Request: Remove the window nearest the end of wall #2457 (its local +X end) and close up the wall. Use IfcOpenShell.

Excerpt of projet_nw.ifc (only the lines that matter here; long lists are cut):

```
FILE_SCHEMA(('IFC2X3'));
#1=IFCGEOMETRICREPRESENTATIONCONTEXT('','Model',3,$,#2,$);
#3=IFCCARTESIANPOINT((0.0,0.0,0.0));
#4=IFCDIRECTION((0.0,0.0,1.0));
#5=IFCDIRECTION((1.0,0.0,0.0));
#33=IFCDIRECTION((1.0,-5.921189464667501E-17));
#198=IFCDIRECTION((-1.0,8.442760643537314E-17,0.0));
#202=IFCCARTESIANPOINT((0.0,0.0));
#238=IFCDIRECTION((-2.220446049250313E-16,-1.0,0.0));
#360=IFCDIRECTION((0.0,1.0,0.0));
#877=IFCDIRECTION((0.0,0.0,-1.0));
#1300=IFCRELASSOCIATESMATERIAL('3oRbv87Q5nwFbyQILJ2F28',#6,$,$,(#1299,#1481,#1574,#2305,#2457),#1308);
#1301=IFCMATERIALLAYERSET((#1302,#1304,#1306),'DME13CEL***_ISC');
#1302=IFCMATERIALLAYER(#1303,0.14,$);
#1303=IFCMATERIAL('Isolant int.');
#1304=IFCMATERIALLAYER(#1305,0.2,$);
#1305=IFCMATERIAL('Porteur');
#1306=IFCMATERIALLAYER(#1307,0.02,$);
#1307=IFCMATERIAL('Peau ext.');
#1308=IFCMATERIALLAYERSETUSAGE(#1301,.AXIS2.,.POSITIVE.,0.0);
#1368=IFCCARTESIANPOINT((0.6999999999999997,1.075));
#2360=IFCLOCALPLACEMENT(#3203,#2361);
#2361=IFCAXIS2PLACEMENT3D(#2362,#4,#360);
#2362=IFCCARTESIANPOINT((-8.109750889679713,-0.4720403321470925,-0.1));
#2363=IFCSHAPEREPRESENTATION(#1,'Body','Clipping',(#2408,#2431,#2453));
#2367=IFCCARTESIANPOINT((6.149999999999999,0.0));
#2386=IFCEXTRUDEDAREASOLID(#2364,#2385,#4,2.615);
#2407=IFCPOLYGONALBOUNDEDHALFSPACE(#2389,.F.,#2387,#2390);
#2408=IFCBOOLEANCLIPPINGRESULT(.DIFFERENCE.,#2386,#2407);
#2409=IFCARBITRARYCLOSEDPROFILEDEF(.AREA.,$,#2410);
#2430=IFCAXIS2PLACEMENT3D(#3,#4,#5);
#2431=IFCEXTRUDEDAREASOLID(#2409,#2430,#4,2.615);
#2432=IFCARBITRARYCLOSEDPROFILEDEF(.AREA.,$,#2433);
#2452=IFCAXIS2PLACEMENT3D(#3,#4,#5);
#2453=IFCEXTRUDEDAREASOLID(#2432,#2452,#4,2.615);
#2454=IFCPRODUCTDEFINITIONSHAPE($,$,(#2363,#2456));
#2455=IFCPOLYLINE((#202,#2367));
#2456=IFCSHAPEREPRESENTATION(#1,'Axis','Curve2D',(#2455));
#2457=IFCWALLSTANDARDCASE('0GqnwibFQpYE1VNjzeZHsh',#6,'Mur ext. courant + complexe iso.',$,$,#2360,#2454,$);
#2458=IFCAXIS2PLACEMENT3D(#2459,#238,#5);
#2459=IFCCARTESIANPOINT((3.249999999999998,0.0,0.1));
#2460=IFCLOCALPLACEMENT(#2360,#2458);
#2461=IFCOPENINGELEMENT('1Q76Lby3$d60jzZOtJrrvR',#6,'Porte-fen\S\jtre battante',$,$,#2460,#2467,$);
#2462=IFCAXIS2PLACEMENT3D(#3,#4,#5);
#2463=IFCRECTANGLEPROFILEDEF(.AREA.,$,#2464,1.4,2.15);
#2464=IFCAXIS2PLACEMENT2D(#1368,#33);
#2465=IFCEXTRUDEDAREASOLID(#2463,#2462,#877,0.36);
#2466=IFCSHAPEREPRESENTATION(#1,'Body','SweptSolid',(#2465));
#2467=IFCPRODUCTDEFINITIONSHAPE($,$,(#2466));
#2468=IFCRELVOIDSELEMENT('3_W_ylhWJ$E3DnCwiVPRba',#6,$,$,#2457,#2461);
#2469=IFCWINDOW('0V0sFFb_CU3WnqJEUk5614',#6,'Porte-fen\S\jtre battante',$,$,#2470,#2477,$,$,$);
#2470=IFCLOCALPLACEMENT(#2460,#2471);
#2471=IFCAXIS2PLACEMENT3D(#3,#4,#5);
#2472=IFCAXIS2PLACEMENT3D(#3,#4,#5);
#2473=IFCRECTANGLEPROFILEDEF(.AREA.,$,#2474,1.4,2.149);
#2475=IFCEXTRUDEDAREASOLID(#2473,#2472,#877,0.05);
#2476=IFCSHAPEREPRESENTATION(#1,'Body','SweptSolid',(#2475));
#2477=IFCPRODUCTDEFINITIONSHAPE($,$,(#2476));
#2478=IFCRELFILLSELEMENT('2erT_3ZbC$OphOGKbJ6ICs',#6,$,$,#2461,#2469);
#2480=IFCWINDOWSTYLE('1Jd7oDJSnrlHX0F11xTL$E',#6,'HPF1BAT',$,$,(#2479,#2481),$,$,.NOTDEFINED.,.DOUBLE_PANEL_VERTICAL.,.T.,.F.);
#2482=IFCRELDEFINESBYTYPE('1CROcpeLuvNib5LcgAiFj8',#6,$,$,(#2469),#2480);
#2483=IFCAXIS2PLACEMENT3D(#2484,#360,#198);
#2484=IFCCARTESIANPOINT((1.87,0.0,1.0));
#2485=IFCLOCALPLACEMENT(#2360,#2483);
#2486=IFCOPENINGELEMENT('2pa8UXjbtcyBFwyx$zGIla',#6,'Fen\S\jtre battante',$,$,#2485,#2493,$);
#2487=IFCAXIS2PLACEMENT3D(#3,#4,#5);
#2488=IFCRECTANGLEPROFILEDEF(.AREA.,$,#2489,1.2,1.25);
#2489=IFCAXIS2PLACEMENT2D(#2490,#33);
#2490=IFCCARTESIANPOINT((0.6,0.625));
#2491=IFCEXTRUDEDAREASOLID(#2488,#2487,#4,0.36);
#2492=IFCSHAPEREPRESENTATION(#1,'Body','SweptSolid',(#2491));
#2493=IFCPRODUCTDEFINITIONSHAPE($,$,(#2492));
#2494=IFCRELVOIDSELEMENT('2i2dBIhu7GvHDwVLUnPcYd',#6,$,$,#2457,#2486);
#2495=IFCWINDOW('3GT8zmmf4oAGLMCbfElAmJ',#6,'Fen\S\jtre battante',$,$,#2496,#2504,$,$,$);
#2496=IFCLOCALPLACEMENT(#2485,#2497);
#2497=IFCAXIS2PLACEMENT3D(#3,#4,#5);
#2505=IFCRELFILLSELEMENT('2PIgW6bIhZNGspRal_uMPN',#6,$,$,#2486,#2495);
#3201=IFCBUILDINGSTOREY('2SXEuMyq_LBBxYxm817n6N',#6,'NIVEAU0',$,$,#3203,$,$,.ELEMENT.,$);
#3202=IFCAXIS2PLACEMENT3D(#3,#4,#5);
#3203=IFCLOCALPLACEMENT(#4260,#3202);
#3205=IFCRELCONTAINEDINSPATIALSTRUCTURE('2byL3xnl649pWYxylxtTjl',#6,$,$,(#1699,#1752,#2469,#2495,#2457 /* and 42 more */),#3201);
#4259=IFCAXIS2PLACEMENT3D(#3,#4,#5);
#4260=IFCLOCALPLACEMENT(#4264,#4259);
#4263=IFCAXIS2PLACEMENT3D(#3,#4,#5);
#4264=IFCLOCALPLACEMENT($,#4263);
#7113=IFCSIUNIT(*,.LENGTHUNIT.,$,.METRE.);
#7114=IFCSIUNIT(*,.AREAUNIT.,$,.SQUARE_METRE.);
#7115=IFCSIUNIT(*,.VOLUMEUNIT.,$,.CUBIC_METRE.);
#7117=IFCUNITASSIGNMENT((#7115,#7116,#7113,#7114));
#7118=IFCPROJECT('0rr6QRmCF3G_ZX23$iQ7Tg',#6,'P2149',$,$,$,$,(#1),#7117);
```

```python
import ifcopenshell
import ifcopenshell.api.feature
import ifcopenshell.api.root
import ifcopenshell.geom
import ifcopenshell.util.shape

model = ifcopenshell.open("projet_nw.ifc")
settings = ifcopenshell.geom.settings()


def volume(element):
    """Net volume in cubic metres, openings subtracted."""
    shape = ifcopenshell.geom.create_shape(settings, element)
    return ifcopenshell.util.shape.get_volume(shape.geometry)


window = model.by_guid("0V0sFFb_CU3WnqJEUk5614")
opening = window.FillsVoids[0].RelatingOpeningElement
wall = opening.VoidsElements[0].RelatingBuildingElement
before = volume(wall)

ifcopenshell.api.root.remove_product(model, product=window)
ifcopenshell.api.feature.remove_feature(model, feature=opening)

after = volume(wall)

print(f"wall volume {before:.3f} -> {after:.3f} m3")

model.write("projet_nw_rev.ifc")
```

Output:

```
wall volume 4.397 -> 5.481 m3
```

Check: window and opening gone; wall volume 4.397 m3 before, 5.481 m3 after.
